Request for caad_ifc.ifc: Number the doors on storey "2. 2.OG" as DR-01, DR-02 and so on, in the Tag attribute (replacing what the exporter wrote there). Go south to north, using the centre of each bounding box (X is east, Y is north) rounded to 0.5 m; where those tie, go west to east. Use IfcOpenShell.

First a look at what the model holds.

```python
import ifcopenshell
import ifcopenshell.util.element
import ifcopenshell.util.placement

model = ifcopenshell.open("caad_ifc.ifc")
print(model.schema)
storey = next(s for s in model.by_type("IfcBuildingStorey") if s.Name == "2. 2.OG")
doors = [e for e in ifcopenshell.util.element.get_decomposition(storey) if e.is_a("IfcDoor")]
for e in sorted(doors, key=lambda e: e.id()):
    origin = ifcopenshell.util.placement.get_local_placement(e.ObjectPlacement)[:3, 3]
    print(e.id(), e.Tag, e.Name, origin.round(2) + 0.0, sep=" | ")
```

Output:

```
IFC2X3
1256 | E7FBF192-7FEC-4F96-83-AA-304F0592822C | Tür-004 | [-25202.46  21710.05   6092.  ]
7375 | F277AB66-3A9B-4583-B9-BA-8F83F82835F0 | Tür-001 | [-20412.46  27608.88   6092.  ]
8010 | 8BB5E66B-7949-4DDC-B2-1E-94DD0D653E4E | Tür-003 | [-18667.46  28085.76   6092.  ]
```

```python
import ifcopenshell
import ifcopenshell.geom
import ifcopenshell.util.element
import ifcopenshell.util.shape

model = ifcopenshell.open("caad_ifc.ifc")
settings = ifcopenshell.geom.settings()
settings.set("use-world-coords", True)


def centre(element):
    shape = ifcopenshell.geom.create_shape(settings, element)
    return ifcopenshell.util.shape.get_bbox_centroid(shape.geometry)


storey = next(s for s in model.by_type("IfcBuildingStorey") if s.Name == "2. 2.OG")
doors = [e for e in ifcopenshell.util.element.get_decomposition(storey) if e.is_a("IfcDoor")]

# Insertion points can sit at a corner or the storey origin, so sort by the geometry (in metres).
centres = {e: centre(e) for e in doors}
doors.sort(key=lambda e: (round(centres[e][1] / 0.5), centres[e][0]))

for i, e in enumerate(doors, start=1):
    number = f"DR-{i:02d}"
    e.Tag = number
    print(e.id(), number)

model.write("caad_ifc-out.ifc")
```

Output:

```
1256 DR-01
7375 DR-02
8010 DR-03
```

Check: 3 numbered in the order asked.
